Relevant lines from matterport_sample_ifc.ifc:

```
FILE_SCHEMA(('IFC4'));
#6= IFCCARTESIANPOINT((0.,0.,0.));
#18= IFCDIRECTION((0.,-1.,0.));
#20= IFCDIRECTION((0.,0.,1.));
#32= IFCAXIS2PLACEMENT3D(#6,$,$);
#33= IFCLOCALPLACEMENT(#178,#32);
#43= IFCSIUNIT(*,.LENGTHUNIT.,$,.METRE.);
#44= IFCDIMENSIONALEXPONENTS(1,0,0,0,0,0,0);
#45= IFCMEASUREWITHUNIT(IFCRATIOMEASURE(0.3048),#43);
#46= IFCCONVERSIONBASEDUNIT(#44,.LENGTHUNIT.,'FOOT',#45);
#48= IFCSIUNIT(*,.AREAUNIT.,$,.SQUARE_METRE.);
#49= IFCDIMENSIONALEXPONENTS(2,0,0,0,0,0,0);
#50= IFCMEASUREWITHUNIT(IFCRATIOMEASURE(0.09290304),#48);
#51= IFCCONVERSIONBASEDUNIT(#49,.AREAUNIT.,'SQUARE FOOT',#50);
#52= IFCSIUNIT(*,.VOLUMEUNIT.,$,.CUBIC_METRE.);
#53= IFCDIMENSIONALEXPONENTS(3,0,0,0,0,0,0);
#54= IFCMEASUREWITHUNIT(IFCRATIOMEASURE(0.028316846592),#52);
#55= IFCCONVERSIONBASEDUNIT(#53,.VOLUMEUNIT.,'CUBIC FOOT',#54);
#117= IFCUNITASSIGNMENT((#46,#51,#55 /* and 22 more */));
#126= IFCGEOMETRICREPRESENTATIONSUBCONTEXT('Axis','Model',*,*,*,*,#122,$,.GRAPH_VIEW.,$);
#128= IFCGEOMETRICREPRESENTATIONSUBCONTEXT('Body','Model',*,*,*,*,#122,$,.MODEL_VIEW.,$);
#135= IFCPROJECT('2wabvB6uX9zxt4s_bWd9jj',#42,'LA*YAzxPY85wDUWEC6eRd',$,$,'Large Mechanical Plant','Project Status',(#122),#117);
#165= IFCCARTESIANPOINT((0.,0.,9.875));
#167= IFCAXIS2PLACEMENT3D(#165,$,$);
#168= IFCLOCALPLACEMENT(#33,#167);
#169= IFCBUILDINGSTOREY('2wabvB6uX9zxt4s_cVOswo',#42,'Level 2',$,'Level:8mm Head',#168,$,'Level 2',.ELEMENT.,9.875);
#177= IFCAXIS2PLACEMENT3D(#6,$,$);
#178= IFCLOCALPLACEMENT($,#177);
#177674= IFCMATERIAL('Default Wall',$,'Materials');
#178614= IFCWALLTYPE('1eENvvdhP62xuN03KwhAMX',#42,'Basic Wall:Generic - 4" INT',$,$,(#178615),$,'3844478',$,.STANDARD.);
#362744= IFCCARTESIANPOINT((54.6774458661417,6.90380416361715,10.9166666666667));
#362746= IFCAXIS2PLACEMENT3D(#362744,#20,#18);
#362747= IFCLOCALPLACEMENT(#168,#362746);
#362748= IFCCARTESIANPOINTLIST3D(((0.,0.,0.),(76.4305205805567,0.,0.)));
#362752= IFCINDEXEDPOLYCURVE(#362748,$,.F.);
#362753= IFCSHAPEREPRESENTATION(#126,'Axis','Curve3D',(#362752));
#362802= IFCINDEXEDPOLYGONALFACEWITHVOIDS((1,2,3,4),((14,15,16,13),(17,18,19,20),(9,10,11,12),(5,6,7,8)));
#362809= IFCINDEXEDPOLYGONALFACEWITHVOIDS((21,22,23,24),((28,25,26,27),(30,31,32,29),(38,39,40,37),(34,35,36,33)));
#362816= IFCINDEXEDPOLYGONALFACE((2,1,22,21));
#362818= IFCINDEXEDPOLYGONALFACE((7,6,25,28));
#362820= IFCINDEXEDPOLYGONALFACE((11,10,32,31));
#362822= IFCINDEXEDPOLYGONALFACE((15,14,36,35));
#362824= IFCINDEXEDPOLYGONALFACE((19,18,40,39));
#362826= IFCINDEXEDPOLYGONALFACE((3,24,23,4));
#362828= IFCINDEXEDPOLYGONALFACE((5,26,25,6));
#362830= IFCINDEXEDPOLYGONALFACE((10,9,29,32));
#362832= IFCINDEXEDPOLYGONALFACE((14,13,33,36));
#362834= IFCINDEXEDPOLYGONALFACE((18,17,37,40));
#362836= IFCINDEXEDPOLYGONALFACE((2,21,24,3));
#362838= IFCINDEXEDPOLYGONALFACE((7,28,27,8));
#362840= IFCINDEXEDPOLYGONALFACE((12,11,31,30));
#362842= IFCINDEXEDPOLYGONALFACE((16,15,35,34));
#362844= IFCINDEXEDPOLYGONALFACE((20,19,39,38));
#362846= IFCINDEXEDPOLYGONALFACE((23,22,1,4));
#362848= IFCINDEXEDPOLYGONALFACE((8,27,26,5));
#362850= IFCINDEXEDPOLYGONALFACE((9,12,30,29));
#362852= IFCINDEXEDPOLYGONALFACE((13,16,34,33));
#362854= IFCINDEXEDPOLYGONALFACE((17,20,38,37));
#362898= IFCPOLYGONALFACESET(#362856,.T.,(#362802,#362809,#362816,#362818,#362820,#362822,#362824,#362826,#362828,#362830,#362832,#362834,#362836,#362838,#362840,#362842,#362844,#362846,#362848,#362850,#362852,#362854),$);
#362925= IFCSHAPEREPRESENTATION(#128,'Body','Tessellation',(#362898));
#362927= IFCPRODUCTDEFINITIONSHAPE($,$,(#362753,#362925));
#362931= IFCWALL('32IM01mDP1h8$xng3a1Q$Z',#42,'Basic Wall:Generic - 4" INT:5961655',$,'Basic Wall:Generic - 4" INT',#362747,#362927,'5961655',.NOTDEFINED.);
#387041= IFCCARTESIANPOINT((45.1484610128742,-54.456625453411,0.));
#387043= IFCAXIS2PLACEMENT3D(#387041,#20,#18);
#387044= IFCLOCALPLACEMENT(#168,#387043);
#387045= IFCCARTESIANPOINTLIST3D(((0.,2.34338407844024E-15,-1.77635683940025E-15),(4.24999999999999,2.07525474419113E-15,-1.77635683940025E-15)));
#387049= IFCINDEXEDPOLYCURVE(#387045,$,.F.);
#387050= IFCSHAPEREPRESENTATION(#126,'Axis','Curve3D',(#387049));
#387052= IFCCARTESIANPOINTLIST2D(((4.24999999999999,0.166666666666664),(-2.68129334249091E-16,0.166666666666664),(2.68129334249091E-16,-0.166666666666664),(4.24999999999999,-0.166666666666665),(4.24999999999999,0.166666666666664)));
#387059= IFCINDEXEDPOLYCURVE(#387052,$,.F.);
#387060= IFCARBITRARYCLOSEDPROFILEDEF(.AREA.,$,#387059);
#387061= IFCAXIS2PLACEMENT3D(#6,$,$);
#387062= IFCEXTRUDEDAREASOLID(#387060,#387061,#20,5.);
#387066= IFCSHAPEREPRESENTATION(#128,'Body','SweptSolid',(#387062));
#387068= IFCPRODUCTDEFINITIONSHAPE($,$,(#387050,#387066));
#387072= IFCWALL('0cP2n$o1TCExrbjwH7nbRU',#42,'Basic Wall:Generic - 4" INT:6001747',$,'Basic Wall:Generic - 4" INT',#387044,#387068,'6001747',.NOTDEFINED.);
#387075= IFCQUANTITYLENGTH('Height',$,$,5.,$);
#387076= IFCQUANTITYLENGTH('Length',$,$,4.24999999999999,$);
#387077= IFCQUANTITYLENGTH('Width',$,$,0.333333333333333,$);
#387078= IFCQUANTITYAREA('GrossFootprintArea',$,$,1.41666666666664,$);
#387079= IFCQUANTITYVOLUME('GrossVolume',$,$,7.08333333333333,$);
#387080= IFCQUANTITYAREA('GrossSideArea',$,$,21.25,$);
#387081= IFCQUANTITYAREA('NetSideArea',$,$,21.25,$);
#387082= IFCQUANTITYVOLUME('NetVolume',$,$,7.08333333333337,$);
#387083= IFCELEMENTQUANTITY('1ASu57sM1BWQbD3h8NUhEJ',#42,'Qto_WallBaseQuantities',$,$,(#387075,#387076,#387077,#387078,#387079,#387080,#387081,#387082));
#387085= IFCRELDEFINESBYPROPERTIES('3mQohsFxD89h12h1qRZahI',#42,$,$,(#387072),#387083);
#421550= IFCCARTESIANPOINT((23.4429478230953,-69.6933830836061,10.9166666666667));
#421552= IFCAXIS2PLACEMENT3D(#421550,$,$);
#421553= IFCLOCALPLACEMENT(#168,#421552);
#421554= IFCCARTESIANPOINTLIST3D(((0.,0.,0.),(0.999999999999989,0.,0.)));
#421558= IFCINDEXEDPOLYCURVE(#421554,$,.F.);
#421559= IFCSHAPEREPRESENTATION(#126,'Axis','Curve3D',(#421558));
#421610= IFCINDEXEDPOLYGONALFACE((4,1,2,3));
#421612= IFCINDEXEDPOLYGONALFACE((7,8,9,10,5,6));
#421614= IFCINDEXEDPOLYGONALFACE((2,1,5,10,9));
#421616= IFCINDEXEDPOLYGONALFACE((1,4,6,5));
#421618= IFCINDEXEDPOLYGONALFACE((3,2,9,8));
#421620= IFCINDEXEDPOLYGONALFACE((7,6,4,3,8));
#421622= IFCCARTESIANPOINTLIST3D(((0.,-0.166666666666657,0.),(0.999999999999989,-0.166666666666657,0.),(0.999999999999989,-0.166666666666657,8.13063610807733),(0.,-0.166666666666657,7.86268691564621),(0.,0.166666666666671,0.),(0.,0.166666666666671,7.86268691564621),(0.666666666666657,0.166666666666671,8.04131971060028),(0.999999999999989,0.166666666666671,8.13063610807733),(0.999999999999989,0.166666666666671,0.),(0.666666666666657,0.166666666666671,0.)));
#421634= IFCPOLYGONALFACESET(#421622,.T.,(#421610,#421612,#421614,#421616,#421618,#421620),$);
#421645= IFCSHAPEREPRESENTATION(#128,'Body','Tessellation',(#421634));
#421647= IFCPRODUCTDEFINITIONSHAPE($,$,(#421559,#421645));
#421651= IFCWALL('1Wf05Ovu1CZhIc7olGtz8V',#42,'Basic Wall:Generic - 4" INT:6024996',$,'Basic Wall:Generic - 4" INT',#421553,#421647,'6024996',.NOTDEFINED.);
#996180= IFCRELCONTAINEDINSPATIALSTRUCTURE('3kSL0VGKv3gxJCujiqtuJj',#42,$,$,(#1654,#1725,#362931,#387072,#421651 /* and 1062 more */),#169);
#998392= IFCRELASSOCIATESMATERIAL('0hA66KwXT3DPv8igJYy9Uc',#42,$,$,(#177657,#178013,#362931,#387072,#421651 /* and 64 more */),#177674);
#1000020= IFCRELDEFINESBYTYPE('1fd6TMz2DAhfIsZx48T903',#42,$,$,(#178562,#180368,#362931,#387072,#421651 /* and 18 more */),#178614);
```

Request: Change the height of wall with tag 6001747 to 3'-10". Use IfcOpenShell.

```python
import ifcopenshell
import ifcopenshell.api.pset
import ifcopenshell.geom
import ifcopenshell.util.element
import ifcopenshell.util.representation
import ifcopenshell.util.shape
import ifcopenshell.util.unit

model = ifcopenshell.open("matterport_sample_ifc.ifc")
unit_scale = ifcopenshell.util.unit.calculate_unit_scale(model)
area_scale = ifcopenshell.util.unit.calculate_unit_scale(model, "AREAUNIT")
volume_scale = ifcopenshell.util.unit.calculate_unit_scale(model, "VOLUMEUNIT")
settings = ifcopenshell.geom.settings()


def volume(element):
    """Net volume in cubic metres, openings subtracted."""
    shape = ifcopenshell.geom.create_shape(settings, element)
    return ifcopenshell.util.shape.get_volume(shape.geometry)


wall = model.by_id(387072)
before = volume(wall)

body = ifcopenshell.util.representation.get_representation(wall, "Model", "Body")
solid = body.Items[0]
old_height = solid.Depth
solid.Depth = 46 * 0.0254 / unit_scale
after = volume(wall)
thickness = 0.1016  # wall thickness in metres

# Update the stored height, areas and volumes.
qto = model.by_id(ifcopenshell.util.element.get_pset(wall, "Qto_WallBaseQuantities", should_inherit=False)["id"])
ifcopenshell.api.pset.edit_qto(model, qto=qto, properties={
    "Height": solid.Depth,
    "GrossVolume": ifcopenshell.util.element.get_pset(wall, "Qto_WallBaseQuantities", "GrossVolume") * solid.Depth / old_height,
    "GrossSideArea": ifcopenshell.util.element.get_pset(wall, "Qto_WallBaseQuantities", "GrossSideArea") * solid.Depth / old_height,
    "NetSideArea": after / thickness / area_scale,
    "NetVolume": after / volume_scale,
})

print(f"height {old_height:g} -> {solid.Depth:g}, volume {before:.3f} -> {after:.3f} m3")

model.write("matterport_sample_ifc_edited.ifc")
```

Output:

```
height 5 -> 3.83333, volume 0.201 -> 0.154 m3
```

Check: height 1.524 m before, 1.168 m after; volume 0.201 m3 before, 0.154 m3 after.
